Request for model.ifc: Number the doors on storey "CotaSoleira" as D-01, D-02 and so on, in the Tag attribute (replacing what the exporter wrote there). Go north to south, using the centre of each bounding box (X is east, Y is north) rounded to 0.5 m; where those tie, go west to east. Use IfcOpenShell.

First a look at what the model holds.

```python
import ifcopenshell
import ifcopenshell.util.element
import ifcopenshell.util.placement

model = ifcopenshell.open("model.ifc")
print(model.schema)
storey = next(s for s in model.by_type("IfcBuildingStorey") if s.Name == "CotaSoleira")
doors = [e for e in ifcopenshell.util.element.get_decomposition(storey) if e.is_a("IfcDoor")]
for e in sorted(doors, key=lambda e: e.id()):
    origin = ifcopenshell.util.placement.get_local_placement(e.ObjectPlacement)[:3, 3]
    print(e.id(), e.Tag, e.Name, origin.round(2) + 0.0, sep=" | ")
```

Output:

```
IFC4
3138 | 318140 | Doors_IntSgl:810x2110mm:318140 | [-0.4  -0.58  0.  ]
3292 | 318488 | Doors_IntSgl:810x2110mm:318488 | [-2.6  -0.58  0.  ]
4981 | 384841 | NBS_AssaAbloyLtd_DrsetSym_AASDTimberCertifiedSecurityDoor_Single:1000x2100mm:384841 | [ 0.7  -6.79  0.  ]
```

```python
import ifcopenshell
import ifcopenshell.geom
import ifcopenshell.util.element
import ifcopenshell.util.shape

model = ifcopenshell.open("model.ifc")
settings = ifcopenshell.geom.settings()
settings.set("use-world-coords", True)


def centre(element):
    shape = ifcopenshell.geom.create_shape(settings, element)
    return ifcopenshell.util.shape.get_bbox_centroid(shape.geometry)


storey = next(s for s in model.by_type("IfcBuildingStorey") if s.Name == "CotaSoleira")
doors = [e for e in ifcopenshell.util.element.get_decomposition(storey) if e.is_a("IfcDoor")]

# Insertion points can sit at a corner or the storey origin, so sort by the geometry (in metres).
centres = {e: centre(e) for e in doors}
doors.sort(key=lambda e: (-round(centres[e][1] / 0.5), centres[e][0]))

for i, e in enumerate(doors, start=1):
    number = f"D-{i:02d}"
    e.Tag = number
    print(e.id(), number)

model.write("model_edited.ifc")
```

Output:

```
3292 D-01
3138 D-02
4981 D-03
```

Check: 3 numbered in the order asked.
